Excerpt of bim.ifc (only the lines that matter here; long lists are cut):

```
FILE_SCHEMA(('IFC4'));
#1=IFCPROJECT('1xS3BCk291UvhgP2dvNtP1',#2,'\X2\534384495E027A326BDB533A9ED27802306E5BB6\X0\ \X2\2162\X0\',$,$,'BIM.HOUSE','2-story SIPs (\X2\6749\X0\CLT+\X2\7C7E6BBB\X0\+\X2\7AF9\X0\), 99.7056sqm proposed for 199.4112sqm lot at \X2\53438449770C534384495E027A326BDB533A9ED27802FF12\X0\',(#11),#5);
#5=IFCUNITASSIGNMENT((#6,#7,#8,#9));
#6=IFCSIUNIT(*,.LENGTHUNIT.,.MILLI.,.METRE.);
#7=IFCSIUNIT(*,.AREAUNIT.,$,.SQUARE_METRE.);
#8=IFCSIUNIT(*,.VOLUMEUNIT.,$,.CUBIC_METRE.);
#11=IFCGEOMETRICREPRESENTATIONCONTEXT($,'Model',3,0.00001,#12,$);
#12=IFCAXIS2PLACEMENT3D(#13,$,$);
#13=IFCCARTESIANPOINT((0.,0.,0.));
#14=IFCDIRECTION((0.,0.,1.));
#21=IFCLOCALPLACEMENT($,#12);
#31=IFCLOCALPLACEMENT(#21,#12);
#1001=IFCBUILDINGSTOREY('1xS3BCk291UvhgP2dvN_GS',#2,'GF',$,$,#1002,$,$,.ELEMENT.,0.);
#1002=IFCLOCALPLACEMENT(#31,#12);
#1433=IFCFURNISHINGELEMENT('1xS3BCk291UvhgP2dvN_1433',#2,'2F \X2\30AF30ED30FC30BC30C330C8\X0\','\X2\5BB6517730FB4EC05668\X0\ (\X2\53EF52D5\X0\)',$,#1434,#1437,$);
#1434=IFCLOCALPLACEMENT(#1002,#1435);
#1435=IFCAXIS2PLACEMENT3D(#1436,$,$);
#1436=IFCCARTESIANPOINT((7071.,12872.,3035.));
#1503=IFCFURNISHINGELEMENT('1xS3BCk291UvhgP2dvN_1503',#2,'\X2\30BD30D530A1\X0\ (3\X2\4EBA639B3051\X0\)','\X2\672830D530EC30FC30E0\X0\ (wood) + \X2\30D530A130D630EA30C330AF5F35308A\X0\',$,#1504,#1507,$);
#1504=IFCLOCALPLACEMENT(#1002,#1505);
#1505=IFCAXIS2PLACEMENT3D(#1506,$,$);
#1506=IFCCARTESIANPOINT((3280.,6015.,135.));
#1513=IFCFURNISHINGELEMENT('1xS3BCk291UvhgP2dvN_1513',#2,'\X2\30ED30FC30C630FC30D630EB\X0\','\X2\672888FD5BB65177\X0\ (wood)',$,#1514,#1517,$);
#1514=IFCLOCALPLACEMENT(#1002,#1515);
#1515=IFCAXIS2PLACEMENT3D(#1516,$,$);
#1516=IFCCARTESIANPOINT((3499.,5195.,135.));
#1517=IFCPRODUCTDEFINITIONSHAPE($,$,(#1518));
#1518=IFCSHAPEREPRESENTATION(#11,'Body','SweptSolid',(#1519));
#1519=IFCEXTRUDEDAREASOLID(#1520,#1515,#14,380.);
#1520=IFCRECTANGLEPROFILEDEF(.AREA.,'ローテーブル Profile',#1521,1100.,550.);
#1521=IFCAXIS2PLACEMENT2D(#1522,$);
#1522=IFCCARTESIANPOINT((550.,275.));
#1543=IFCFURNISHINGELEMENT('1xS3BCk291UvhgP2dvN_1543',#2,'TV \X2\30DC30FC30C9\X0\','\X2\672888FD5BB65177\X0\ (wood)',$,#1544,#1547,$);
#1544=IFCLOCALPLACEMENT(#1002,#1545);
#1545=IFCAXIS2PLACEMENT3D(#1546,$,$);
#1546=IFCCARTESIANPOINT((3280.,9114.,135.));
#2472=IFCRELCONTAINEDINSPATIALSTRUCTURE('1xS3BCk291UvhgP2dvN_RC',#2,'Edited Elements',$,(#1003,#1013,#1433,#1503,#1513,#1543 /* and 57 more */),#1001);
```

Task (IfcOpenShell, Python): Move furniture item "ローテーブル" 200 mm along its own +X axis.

```python
import ifcopenshell
import ifcopenshell.api.geometry
import ifcopenshell.util.placement

model = ifcopenshell.open("bim.ifc")

item = model.by_guid("1xS3BCk291UvhgP2dvN_1513")
matrix = ifcopenshell.util.placement.get_local_placement(item.ObjectPlacement)
matrix[:3, 3] += matrix[:3, 0] * 200.0
ifcopenshell.api.geometry.edit_object_placement(model, product=item, matrix=matrix, is_si=False)

print(ifcopenshell.util.placement.get_local_placement(item.ObjectPlacement).round(3) + 0.0)

model.write("bim_edited.ifc")
```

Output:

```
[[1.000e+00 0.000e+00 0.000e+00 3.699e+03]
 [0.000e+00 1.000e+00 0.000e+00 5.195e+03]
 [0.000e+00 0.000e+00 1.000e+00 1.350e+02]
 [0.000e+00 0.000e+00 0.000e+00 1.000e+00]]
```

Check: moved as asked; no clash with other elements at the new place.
